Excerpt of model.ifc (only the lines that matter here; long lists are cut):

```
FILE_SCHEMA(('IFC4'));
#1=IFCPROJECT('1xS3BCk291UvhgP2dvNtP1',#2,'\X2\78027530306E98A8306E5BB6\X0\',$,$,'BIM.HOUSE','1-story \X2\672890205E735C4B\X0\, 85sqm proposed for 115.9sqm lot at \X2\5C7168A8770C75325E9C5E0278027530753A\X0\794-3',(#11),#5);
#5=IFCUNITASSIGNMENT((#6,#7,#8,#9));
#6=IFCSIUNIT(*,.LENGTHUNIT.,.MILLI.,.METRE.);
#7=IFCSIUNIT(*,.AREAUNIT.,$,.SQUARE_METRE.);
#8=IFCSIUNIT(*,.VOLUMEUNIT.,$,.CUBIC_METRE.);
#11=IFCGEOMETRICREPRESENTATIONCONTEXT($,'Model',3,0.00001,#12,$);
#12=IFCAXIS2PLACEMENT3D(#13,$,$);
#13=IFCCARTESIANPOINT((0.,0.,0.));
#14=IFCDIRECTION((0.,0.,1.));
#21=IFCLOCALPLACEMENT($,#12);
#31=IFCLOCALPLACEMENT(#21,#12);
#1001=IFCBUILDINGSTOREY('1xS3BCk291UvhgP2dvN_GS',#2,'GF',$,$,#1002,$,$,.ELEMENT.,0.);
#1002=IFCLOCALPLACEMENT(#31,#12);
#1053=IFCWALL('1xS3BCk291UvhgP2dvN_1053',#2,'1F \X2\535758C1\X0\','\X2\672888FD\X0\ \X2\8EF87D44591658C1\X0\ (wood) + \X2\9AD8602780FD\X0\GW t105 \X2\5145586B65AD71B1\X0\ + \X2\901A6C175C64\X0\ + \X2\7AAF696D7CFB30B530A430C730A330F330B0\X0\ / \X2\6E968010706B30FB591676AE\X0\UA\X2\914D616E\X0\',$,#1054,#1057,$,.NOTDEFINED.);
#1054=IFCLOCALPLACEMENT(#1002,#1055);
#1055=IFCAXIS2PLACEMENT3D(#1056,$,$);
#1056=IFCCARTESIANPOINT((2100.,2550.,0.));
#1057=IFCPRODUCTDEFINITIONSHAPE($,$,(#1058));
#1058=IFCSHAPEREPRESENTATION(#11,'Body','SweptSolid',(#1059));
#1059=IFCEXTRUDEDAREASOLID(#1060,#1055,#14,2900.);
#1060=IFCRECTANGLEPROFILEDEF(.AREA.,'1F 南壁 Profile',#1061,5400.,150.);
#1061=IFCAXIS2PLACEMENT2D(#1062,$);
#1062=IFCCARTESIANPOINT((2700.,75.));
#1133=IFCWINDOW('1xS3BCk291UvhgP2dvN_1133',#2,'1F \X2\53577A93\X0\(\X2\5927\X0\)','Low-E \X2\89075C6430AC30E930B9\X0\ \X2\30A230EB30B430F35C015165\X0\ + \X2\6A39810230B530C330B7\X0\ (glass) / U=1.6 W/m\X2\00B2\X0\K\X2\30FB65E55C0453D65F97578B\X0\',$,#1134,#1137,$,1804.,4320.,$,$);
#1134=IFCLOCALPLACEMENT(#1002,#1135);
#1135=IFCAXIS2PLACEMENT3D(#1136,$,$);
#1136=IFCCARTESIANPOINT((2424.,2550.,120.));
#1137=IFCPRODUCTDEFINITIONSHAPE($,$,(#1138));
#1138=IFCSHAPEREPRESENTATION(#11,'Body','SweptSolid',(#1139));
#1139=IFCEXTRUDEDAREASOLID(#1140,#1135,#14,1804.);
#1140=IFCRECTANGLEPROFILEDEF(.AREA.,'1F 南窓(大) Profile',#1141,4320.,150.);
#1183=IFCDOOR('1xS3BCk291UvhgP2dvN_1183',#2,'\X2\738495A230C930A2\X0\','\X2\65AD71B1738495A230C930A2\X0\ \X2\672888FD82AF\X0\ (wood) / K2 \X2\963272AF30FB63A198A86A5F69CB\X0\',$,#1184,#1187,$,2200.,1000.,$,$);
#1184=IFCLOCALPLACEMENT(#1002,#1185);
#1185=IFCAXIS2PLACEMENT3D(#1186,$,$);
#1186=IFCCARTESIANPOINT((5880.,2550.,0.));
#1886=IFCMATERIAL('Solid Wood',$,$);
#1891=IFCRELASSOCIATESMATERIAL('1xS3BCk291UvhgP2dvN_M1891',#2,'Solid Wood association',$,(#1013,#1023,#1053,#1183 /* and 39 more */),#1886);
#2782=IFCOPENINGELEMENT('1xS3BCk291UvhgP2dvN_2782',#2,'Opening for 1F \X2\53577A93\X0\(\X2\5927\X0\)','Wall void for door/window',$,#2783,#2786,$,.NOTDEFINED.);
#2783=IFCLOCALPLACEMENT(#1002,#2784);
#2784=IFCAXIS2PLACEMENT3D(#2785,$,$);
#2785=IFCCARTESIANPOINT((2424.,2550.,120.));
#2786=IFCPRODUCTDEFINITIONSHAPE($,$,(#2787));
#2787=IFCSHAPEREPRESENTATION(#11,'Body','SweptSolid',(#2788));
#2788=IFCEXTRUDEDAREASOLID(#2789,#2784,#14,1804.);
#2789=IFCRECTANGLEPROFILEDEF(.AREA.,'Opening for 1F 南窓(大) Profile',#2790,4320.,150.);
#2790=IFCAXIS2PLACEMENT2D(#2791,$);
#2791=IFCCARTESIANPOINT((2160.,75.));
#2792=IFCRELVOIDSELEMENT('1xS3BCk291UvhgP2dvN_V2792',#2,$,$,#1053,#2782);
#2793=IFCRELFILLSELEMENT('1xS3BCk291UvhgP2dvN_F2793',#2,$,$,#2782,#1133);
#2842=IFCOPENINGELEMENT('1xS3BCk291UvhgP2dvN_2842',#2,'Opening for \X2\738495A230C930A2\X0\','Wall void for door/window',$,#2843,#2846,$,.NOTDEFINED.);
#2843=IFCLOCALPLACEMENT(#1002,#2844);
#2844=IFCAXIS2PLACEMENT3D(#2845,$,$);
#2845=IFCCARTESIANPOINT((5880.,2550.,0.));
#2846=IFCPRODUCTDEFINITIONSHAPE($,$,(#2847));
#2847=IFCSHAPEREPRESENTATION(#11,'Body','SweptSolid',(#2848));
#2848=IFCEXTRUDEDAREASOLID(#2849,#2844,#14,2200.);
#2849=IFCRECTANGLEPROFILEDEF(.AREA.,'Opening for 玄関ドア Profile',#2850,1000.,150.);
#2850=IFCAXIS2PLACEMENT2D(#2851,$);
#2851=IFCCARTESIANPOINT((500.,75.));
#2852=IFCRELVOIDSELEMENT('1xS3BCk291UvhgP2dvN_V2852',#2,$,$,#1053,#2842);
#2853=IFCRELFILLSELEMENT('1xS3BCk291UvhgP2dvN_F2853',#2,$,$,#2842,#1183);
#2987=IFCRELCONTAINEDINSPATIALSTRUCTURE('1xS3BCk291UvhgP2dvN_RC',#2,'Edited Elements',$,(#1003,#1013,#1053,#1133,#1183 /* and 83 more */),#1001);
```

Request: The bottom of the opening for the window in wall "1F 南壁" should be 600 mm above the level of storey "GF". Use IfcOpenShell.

```python
import numpy as np
import ifcopenshell
import ifcopenshell.api.geometry
import ifcopenshell.geom
import ifcopenshell.util.element
import ifcopenshell.util.placement
import ifcopenshell.util.shape
import ifcopenshell.util.unit

model = ifcopenshell.open("model.ifc")
unit_scale = ifcopenshell.util.unit.calculate_unit_scale(model)

window = model.by_guid("1xS3BCk291UvhgP2dvN_1133")
opening = window.FillsVoids[0].RelatingOpeningElement
storey = ifcopenshell.util.element.get_container(window, ifc_class="IfcBuildingStorey")
level = ifcopenshell.util.placement.get_local_placement(storey.ObjectPlacement)[2, 3]

# The opening's origin need not be at the sill, so measure its lowest point.
shape = ifcopenshell.geom.create_shape(ifcopenshell.geom.settings(), opening)
bottom = ifcopenshell.util.shape.get_shape_bottom_elevation(shape, shape.geometry) / unit_scale
dz = level + 600.0 - bottom

shift = np.array([0.0, 0.0, dz])
# The window is not placed relative to its opening, so move both.
for product in (opening, window):
    matrix = ifcopenshell.util.placement.get_local_placement(product.ObjectPlacement)
    matrix[:3, 3] += shift
    ifcopenshell.api.geometry.edit_object_placement(model, product=product, matrix=matrix, is_si=False)

print(f"moved by {dz * unit_scale:+.3f} m")

model.write("model_edited.ifc")
```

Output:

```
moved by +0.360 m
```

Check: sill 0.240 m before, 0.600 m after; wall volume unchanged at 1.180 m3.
